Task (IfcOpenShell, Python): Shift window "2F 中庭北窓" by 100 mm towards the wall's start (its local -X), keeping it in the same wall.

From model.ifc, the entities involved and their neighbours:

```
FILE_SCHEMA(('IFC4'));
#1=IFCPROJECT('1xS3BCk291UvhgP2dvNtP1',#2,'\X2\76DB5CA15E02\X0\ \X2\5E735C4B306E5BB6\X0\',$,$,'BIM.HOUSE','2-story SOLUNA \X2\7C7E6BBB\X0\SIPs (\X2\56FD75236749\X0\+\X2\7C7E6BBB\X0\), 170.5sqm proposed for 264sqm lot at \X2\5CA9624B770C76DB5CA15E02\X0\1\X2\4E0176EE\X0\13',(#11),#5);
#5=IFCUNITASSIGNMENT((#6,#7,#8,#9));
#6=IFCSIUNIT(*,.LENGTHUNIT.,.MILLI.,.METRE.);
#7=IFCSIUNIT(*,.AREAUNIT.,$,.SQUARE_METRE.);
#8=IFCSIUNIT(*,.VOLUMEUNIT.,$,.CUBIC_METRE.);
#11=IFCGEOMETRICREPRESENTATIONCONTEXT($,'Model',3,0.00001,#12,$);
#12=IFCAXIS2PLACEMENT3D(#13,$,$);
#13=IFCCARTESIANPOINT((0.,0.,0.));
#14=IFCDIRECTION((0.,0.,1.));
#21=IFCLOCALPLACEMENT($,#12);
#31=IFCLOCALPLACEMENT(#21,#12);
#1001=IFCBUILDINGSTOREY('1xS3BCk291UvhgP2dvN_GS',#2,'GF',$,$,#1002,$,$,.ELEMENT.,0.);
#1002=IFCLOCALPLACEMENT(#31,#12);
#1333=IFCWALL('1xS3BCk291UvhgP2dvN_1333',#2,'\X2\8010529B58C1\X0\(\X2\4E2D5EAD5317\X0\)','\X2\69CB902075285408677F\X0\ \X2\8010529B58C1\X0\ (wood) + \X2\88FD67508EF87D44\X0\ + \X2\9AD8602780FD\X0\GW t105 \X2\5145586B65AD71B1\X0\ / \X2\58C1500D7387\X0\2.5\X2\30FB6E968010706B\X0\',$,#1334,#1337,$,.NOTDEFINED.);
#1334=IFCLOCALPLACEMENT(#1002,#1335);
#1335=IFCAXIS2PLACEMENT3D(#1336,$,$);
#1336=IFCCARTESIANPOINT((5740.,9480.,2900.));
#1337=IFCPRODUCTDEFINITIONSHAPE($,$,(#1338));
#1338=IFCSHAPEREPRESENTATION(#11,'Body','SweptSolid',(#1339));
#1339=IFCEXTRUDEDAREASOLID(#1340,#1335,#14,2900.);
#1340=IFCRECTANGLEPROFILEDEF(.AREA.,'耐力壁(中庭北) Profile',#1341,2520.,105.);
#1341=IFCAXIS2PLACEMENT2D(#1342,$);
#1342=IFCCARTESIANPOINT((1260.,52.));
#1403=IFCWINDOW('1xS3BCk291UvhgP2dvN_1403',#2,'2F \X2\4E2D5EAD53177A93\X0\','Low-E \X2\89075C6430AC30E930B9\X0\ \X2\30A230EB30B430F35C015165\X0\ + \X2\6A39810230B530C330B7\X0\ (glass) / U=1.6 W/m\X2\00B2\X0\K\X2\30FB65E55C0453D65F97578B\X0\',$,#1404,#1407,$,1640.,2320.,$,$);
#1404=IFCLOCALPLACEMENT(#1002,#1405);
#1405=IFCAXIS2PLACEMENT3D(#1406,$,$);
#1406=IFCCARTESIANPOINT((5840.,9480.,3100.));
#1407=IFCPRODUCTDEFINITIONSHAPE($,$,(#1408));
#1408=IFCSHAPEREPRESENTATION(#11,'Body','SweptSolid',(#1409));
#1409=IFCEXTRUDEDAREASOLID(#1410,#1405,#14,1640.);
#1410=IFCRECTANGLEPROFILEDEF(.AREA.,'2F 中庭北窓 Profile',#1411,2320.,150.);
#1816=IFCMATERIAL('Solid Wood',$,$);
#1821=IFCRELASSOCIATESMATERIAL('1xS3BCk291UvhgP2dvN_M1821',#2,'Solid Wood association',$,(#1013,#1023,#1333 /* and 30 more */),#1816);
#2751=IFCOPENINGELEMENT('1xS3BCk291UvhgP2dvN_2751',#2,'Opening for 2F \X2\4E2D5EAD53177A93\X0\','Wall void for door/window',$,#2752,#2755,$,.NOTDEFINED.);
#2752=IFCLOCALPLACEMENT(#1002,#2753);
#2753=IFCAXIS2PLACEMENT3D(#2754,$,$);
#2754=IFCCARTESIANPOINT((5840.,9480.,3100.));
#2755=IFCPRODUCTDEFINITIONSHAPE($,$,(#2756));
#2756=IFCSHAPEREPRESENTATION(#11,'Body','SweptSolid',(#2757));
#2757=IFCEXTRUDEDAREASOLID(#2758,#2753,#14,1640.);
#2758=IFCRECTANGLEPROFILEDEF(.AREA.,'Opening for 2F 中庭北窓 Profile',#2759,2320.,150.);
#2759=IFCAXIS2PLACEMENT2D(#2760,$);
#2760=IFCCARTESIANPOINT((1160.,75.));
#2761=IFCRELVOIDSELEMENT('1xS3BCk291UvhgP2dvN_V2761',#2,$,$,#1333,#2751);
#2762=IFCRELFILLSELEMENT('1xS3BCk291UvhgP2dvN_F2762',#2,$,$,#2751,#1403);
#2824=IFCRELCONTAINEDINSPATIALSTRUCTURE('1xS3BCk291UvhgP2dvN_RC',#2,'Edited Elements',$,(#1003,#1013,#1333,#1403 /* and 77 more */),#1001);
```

```python
import ifcopenshell
import ifcopenshell.api.geometry
import ifcopenshell.util.placement

model = ifcopenshell.open("model.ifc")

window = model.by_guid("1xS3BCk291UvhgP2dvN_1403")
opening = window.FillsVoids[0].RelatingOpeningElement
wall = opening.VoidsElements[0].RelatingBuildingElement

wall_matrix = ifcopenshell.util.placement.get_local_placement(wall.ObjectPlacement)
shift = wall_matrix[:3, 0] * -100.0
before = ifcopenshell.util.placement.get_local_placement(window.ObjectPlacement)[:3, 3].copy()

# The window is not placed relative to its opening, so move both.
for product in (opening, window):
    matrix = ifcopenshell.util.placement.get_local_placement(product.ObjectPlacement)
    matrix[:3, 3] += shift
    ifcopenshell.api.geometry.edit_object_placement(model, product=product, matrix=matrix, is_si=False)

after = ifcopenshell.util.placement.get_local_placement(window.ObjectPlacement)[:3, 3]
print("window moved by", (after - before).round(3) + 0.0)

model.write("model_edited.ifc")
```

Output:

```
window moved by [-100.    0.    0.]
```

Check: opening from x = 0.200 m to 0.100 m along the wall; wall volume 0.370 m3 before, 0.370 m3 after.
